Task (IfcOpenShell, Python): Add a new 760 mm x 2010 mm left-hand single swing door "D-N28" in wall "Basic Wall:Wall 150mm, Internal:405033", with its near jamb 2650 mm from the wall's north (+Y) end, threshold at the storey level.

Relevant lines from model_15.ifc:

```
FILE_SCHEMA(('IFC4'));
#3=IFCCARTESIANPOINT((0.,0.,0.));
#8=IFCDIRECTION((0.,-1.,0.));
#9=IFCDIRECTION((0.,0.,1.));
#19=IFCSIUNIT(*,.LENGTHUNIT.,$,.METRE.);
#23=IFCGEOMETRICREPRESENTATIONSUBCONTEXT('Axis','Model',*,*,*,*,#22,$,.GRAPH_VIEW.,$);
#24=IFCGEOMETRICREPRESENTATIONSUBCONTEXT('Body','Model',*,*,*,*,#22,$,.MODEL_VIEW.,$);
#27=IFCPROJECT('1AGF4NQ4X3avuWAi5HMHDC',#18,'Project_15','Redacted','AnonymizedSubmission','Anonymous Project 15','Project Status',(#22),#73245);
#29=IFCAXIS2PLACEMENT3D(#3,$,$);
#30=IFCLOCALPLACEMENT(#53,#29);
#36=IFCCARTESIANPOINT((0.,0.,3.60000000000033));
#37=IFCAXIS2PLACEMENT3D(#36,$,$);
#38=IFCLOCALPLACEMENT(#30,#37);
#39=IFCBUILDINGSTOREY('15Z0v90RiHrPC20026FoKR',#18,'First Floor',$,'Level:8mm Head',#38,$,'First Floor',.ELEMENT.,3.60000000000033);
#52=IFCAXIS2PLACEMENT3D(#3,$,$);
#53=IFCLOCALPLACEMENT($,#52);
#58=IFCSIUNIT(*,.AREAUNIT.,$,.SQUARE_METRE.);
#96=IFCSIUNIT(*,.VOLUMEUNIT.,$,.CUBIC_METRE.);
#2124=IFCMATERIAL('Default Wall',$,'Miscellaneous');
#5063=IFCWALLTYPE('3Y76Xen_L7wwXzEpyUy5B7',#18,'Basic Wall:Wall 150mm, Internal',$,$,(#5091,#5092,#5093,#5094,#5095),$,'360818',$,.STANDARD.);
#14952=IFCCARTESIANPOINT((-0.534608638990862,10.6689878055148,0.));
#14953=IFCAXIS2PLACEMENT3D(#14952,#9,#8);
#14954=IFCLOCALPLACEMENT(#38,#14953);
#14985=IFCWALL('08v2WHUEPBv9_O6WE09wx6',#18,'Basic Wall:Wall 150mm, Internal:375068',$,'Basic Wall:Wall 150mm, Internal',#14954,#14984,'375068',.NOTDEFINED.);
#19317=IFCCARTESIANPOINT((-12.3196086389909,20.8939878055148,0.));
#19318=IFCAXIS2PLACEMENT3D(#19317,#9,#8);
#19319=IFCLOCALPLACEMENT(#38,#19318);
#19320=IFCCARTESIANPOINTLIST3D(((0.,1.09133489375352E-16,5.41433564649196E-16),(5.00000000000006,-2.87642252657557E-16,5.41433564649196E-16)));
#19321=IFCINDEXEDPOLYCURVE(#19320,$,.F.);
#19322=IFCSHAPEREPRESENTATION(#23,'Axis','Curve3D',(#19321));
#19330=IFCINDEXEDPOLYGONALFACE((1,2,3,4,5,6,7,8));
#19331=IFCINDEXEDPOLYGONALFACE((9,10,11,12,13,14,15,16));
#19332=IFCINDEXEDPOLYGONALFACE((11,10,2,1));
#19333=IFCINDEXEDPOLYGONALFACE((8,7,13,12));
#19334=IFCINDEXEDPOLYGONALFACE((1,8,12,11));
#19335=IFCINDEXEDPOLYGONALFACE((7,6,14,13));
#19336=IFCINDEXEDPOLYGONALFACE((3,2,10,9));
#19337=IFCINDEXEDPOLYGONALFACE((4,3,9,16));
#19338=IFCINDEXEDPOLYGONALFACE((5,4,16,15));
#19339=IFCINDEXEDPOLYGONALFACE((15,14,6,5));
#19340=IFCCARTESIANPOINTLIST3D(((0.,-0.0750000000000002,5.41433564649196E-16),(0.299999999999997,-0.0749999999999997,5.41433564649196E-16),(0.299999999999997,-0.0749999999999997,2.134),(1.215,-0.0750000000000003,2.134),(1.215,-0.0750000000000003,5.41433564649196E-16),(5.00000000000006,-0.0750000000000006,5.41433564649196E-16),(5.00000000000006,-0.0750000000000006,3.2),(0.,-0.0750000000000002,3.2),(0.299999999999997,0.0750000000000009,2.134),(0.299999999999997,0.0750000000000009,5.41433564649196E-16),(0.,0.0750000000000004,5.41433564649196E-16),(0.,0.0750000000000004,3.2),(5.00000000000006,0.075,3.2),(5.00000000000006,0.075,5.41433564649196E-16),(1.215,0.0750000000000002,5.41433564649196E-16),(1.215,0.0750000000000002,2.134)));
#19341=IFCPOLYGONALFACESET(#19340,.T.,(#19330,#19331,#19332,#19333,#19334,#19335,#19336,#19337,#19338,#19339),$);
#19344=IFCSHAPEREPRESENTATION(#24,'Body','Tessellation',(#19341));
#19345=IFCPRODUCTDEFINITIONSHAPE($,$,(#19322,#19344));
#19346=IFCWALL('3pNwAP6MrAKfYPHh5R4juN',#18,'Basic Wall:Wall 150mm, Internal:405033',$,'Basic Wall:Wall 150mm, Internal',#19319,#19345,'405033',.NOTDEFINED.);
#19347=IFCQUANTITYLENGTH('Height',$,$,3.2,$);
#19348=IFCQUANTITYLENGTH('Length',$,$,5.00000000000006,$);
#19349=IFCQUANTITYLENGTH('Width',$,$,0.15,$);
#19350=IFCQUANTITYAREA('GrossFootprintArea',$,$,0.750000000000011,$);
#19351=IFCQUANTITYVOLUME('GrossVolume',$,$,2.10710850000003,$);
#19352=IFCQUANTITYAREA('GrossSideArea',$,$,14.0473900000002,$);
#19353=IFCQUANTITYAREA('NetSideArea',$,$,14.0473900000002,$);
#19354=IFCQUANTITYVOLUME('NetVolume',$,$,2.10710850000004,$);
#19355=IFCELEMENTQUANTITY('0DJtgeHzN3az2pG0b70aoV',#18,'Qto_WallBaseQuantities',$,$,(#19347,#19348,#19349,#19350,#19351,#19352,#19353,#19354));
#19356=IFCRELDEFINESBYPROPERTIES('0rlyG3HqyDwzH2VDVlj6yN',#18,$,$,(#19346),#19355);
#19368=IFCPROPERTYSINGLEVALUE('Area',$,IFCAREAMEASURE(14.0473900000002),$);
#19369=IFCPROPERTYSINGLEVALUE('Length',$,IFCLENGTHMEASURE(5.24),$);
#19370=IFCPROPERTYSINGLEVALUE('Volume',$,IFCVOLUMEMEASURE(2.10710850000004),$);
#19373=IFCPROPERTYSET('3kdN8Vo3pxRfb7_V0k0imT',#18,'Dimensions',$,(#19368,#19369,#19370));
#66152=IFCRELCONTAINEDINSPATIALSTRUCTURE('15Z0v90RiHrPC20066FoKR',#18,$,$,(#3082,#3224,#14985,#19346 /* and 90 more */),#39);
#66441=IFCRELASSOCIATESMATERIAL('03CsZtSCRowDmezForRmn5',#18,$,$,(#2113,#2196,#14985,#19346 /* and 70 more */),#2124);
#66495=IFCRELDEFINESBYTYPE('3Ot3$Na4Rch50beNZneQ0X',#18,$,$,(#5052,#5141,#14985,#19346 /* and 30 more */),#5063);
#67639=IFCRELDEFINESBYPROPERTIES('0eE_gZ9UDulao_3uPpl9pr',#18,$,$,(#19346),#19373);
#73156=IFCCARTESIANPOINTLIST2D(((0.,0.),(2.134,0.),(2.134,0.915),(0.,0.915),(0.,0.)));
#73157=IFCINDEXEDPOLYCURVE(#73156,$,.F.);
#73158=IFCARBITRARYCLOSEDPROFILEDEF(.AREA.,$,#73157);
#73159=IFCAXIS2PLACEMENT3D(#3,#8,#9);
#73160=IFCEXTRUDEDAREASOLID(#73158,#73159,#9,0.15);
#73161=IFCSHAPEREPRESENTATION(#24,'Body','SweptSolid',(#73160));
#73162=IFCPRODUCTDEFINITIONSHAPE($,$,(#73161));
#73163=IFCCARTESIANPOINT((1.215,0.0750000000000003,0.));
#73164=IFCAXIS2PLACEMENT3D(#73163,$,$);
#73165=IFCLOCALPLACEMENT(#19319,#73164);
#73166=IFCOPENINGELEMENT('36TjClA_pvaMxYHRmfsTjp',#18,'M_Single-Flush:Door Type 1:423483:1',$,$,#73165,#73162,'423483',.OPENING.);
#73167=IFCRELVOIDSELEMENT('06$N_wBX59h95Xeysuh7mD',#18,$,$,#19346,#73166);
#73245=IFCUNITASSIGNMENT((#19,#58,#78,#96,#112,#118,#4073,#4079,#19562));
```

```python
import numpy as np
import ifcopenshell
import ifcopenshell.api.feature
import ifcopenshell.api.geometry
import ifcopenshell.api.pset
import ifcopenshell.api.root
import ifcopenshell.api.spatial
import ifcopenshell.geom
import ifcopenshell.util.element
import ifcopenshell.util.placement
import ifcopenshell.util.representation
import ifcopenshell.util.shape
import ifcopenshell.util.unit

model = ifcopenshell.open("model_15.ifc")
unit_scale = ifcopenshell.util.unit.calculate_unit_scale(model)
area_scale = ifcopenshell.util.unit.calculate_unit_scale(model, "AREAUNIT")
volume_scale = ifcopenshell.util.unit.calculate_unit_scale(model, "VOLUMEUNIT")
settings = ifcopenshell.geom.settings()


def volume(element):
    """Net volume in cubic metres, openings subtracted."""
    shape = ifcopenshell.geom.create_shape(settings, element)
    return ifcopenshell.util.shape.get_volume(shape.geometry)


wall = model.by_id(19346)
storey = ifcopenshell.util.element.get_container(wall, ifc_class="IfcBuildingStorey")
context = ifcopenshell.util.representation.get_context(model, "Model", "Body", "MODEL_VIEW")
before = volume(wall)

width, height, from_end, sill = 0.76, 2.01, 2.65, 0.0  # metres

# The wall runs along its own X axis, and the end named is its -X end.
wall_shape = ifcopenshell.geom.create_shape(settings, wall)
x, y, z = ifcopenshell.util.shape.get_vertices(wall_shape.geometry).T
start = x.min() + from_end
face, thickness = float(y.min()), float(y.max() - y.min())
wall_matrix = ifcopenshell.util.placement.get_local_placement(wall.ObjectPlacement)
level = ifcopenshell.util.placement.get_local_placement(storey.ObjectPlacement)[2, 3]


def in_wall(x, y):
    """Placement at x, y metres in the wall's axes, at sill height."""
    matrix = wall_matrix.copy()
    matrix[:, 3] = wall_matrix @ np.array([x / unit_scale, y / unit_scale, 0.0, 1.0])
    matrix[2, 3] = level + sill / unit_scale
    return matrix


# Opening: a box that overshoots both wall faces by 50 mm.
opening = ifcopenshell.api.root.create_entity(model, ifc_class="IfcOpeningElement", predefined_type="OPENING")
box = ifcopenshell.api.geometry.add_wall_representation(
    model, context=context, length=width, height=height, thickness=thickness + 0.1
)
ifcopenshell.api.geometry.assign_representation(model, product=opening, representation=box)
ifcopenshell.api.geometry.edit_object_placement(model, product=opening, matrix=in_wall(start, face - 0.05), is_si=False)
ifcopenshell.api.feature.add_feature(model, feature=opening, element=wall)

door = ifcopenshell.api.root.create_entity(model, ifc_class="IfcDoor", name="D-N28", predefined_type="DOOR")
door.OverallWidth, door.OverallHeight = width / unit_scale, height / unit_scale
door.OperationType = "SINGLE_SWING_LEFT"
body = ifcopenshell.api.geometry.add_door_representation(
    model,
    context=context,
    overall_width=door.OverallWidth,
    overall_height=door.OverallHeight,
    operation_type="SINGLE_SWING_LEFT",
    lining_properties={"LiningDepth": thickness / unit_scale, "ThresholdDepth": thickness / unit_scale},
)
ifcopenshell.api.geometry.assign_representation(model, product=door, representation=body)
ifcopenshell.api.spatial.assign_container(model, products=[door], relating_structure=storey)
ifcopenshell.api.feature.add_filling(model, opening=opening, element=door)

# The lining spans the wall, so the door starts at the wall face.
ifcopenshell.api.geometry.edit_object_placement(model, product=door, matrix=in_wall(start, face), is_si=False)

after = volume(wall)

# Update the wall's stored quantities.
qto = model.by_id(ifcopenshell.util.element.get_pset(wall, "Qto_WallBaseQuantities", should_inherit=False)["id"])
ifcopenshell.api.pset.edit_qto(model, qto=qto, properties={
    "NetSideArea": after / thickness / area_scale,
    "NetVolume": after / volume_scale,
})
pset = model.by_id(ifcopenshell.util.element.get_pset(wall, "Dimensions", should_inherit=False)["id"])
ifcopenshell.api.pset.edit_pset(model, pset=pset, properties={
    "Area": model.create_entity("IfcAreaMeasure", after / thickness / area_scale),
    "Volume": model.create_entity("IfcVolumeMeasure", after / volume_scale),
})

print(f"wall volume {before:.3f} -> {after:.3f} m3")

model.write("model_15_rev.ifc")
```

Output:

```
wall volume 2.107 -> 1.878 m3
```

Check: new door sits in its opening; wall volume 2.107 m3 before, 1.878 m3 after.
